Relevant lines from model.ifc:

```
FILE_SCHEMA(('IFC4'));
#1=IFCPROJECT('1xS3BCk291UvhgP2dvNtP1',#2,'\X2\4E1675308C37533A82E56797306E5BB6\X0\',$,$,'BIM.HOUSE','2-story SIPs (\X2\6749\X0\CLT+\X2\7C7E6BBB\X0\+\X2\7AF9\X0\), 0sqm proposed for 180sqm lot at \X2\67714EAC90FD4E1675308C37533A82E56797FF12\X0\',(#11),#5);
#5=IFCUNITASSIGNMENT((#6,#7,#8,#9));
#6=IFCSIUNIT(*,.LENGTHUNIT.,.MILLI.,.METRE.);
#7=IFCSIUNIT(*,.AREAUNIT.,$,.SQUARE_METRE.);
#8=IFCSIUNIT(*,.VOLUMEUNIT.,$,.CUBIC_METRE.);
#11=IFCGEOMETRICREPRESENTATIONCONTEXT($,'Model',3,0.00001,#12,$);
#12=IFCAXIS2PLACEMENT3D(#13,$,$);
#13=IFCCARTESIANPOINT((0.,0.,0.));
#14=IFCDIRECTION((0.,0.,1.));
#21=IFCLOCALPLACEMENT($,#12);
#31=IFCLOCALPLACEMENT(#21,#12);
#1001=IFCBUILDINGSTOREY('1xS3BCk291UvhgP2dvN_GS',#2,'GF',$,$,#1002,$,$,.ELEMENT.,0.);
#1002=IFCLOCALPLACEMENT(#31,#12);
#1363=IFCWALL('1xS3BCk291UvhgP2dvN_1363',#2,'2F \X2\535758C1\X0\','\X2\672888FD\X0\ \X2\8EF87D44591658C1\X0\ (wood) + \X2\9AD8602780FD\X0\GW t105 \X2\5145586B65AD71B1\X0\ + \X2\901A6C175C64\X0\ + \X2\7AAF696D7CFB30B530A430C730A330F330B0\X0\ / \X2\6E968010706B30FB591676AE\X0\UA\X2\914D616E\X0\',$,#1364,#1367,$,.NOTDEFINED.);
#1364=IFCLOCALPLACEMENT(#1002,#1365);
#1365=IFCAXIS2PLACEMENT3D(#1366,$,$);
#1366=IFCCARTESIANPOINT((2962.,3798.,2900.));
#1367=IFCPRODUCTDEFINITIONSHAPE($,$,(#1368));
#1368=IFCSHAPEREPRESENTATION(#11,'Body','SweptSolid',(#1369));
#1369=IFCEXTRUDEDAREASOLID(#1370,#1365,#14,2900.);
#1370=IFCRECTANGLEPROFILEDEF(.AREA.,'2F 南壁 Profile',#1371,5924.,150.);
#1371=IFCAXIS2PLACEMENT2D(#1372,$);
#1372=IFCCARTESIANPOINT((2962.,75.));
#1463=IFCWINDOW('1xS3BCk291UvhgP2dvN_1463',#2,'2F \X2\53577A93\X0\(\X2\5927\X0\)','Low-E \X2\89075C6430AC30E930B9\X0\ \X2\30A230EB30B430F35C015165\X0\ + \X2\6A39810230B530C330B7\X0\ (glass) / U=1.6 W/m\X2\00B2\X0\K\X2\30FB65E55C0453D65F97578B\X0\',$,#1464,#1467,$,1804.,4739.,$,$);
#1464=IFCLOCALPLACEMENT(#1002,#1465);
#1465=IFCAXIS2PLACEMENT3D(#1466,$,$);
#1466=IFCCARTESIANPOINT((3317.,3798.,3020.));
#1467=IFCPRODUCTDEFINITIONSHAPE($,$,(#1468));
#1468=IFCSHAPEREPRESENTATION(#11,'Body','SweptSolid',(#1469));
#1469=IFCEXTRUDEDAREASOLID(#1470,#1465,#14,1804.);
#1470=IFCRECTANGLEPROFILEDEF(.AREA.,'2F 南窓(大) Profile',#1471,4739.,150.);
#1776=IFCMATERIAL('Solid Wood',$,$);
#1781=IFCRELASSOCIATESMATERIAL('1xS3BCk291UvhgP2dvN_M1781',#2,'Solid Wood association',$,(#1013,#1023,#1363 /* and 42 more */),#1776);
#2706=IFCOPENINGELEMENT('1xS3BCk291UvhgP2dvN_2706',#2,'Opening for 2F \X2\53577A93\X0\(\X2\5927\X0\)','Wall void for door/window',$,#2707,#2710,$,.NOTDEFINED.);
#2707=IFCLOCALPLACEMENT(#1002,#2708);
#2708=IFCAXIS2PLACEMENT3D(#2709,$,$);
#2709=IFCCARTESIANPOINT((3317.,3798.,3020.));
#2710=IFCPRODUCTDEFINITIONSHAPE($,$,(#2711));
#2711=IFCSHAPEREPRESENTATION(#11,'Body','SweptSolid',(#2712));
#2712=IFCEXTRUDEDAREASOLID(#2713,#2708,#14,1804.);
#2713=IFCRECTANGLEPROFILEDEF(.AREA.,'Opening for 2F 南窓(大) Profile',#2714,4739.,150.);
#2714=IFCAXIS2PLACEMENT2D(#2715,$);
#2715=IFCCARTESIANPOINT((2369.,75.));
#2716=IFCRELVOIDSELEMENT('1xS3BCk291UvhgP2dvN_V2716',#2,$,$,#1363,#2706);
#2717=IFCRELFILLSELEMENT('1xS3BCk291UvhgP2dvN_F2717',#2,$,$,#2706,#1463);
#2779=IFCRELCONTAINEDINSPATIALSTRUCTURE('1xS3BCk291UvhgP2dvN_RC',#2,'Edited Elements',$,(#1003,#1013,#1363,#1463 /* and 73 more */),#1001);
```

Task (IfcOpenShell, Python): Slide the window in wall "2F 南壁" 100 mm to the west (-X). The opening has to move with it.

```python
import ifcopenshell
import ifcopenshell.api.geometry
import ifcopenshell.util.placement
import ifcopenshell.util.unit

model = ifcopenshell.open("model.ifc")
unit_scale = ifcopenshell.util.unit.calculate_unit_scale(model)

window = model.by_guid("1xS3BCk291UvhgP2dvN_1463")
opening = window.FillsVoids[0].RelatingOpeningElement
wall = opening.VoidsElements[0].RelatingBuildingElement

wall_matrix = ifcopenshell.util.placement.get_local_placement(wall.ObjectPlacement)
shift = wall_matrix[:3, 0] * -0.1 / unit_scale
before = ifcopenshell.util.placement.get_local_placement(window.ObjectPlacement)[:3, 3].copy()

# The window is not placed relative to its opening, so move both.
for product in (opening, window):
    matrix = ifcopenshell.util.placement.get_local_placement(product.ObjectPlacement)
    matrix[:3, 3] += shift
    ifcopenshell.api.geometry.edit_object_placement(model, product=product, matrix=matrix, is_si=False)

after = ifcopenshell.util.placement.get_local_placement(window.ObjectPlacement)[:3, 3]
print("window moved by", (after - before).round(3) + 0.0)

model.write("model_rev.ifc")
```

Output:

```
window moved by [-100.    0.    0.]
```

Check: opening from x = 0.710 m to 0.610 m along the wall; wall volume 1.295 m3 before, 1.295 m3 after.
